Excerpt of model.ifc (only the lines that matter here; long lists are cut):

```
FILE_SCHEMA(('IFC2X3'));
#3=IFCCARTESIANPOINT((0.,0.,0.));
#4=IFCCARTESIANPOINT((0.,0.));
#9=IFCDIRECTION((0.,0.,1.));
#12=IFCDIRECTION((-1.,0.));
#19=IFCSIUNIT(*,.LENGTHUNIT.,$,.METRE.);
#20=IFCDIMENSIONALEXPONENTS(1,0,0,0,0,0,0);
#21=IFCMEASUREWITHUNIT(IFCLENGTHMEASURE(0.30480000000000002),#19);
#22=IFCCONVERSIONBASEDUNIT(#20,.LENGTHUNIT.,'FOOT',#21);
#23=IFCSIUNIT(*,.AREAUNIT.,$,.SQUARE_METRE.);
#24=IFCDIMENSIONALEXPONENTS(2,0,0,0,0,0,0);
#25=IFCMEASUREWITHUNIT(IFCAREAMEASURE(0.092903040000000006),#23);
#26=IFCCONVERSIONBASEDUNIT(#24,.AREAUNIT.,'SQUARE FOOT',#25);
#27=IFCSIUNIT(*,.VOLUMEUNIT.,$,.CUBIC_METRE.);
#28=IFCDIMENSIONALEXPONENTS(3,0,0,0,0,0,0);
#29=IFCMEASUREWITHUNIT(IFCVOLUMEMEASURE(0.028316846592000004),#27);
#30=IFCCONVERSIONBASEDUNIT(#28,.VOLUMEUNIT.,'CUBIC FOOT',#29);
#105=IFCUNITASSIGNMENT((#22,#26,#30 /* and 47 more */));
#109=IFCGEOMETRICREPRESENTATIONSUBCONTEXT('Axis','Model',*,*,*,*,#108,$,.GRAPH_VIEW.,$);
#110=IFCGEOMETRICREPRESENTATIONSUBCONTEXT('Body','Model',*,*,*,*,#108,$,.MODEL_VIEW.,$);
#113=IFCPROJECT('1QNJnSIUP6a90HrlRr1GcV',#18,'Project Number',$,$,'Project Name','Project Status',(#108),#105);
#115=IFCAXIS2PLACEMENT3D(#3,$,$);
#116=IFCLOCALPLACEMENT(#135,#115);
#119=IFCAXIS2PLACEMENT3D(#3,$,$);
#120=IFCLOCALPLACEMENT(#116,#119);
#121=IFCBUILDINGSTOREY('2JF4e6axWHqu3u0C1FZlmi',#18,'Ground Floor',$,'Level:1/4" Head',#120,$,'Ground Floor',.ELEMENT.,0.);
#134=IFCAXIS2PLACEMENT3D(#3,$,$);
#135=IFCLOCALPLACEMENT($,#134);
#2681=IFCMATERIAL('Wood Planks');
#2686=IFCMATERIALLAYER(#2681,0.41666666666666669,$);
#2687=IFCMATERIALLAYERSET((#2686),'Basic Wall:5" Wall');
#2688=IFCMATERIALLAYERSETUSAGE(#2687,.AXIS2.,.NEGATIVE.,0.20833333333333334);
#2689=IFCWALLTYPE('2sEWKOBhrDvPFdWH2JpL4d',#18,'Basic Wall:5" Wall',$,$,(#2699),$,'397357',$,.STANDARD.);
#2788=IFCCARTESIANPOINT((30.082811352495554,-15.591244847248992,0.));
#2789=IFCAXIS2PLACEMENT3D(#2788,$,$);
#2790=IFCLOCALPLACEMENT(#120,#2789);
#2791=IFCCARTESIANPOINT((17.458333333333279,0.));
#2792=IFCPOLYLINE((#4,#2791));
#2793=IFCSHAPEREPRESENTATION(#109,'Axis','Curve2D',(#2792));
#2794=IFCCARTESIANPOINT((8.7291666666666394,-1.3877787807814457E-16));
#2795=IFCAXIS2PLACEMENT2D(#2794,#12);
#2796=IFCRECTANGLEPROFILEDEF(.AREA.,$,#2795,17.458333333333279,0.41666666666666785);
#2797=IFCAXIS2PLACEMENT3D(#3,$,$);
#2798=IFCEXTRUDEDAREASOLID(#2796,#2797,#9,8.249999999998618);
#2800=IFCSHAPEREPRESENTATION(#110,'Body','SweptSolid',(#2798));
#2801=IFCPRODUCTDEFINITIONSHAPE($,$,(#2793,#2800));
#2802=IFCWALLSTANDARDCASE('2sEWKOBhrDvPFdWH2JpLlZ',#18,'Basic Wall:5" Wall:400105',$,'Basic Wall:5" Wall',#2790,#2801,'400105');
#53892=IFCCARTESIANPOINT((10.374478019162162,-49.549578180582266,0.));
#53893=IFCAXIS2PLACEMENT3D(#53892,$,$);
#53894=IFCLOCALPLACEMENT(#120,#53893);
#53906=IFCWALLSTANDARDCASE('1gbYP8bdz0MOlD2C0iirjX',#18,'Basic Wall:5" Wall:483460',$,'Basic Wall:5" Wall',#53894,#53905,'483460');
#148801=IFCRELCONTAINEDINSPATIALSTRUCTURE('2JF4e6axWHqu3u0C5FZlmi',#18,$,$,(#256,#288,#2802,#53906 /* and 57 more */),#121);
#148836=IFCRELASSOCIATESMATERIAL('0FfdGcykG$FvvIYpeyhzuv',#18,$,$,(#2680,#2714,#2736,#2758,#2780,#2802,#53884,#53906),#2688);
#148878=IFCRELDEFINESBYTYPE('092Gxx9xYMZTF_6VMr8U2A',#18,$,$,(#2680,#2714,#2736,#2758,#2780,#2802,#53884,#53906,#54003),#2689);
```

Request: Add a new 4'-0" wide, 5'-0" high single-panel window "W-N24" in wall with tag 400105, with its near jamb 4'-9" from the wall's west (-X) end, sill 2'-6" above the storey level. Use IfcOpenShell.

```python
import numpy as np
import ifcopenshell
import ifcopenshell.api.feature
import ifcopenshell.api.geometry
import ifcopenshell.api.root
import ifcopenshell.api.spatial
import ifcopenshell.api.type
import ifcopenshell.geom
import ifcopenshell.util.element
import ifcopenshell.util.placement
import ifcopenshell.util.representation
import ifcopenshell.util.shape
import ifcopenshell.util.unit

model = ifcopenshell.open("model.ifc")
unit_scale = ifcopenshell.util.unit.calculate_unit_scale(model)
settings = ifcopenshell.geom.settings()


def volume(element):
    """Net volume in cubic metres, openings subtracted."""
    shape = ifcopenshell.geom.create_shape(settings, element)
    return ifcopenshell.util.shape.get_volume(shape.geometry)


wall = model.by_id(2802)
storey = ifcopenshell.util.element.get_container(wall, ifc_class="IfcBuildingStorey")
context = ifcopenshell.util.representation.get_context(model, "Model", "Body", "MODEL_VIEW")
before = volume(wall)

width, height, from_end, sill = 1.2192, 1.524, 1.4478, 0.762  # metres

# The wall runs along its own X axis, and the end named is its -X end.
wall_shape = ifcopenshell.geom.create_shape(settings, wall)
x, y, z = ifcopenshell.util.shape.get_vertices(wall_shape.geometry).T
start = x.min() + from_end
face, thickness = float(y.min()), float(y.max() - y.min())
wall_matrix = ifcopenshell.util.placement.get_local_placement(wall.ObjectPlacement)
level = ifcopenshell.util.placement.get_local_placement(storey.ObjectPlacement)[2, 3]


def in_wall(x, y):
    """Placement at x, y metres in the wall's axes, at sill height."""
    matrix = wall_matrix.copy()
    matrix[:, 3] = wall_matrix @ np.array([x / unit_scale, y / unit_scale, 0.0, 1.0])
    matrix[2, 3] = level + sill / unit_scale
    return matrix


# Opening: a box that overshoots both wall faces by 50 mm.
opening = ifcopenshell.api.root.create_entity(model, ifc_class="IfcOpeningElement")
box = ifcopenshell.api.geometry.add_wall_representation(
    model, context=context, length=width, height=height, thickness=thickness + 0.1
)
ifcopenshell.api.geometry.assign_representation(model, product=opening, representation=box)
ifcopenshell.api.geometry.edit_object_placement(model, product=opening, matrix=in_wall(start, face - 0.05), is_si=False)
ifcopenshell.api.feature.add_feature(model, feature=opening, element=wall)

window = ifcopenshell.api.root.create_entity(model, ifc_class="IfcWindow", name="W-N24")
window.OverallWidth, window.OverallHeight = width / unit_scale, height / unit_scale
body = ifcopenshell.api.geometry.add_window_representation(
    model,
    context=context,
    overall_width=window.OverallWidth,
    overall_height=window.OverallHeight,
    partition_type="SINGLE_PANEL",
)
ifcopenshell.api.geometry.assign_representation(model, product=window, representation=body)
ifcopenshell.api.spatial.assign_container(model, products=[window], relating_structure=storey)
fills = ifcopenshell.api.feature.add_filling(model, opening=opening, element=window)
fills.OwnerHistory = window.OwnerHistory  # required in IFC2X3

# IFC2X3 keeps the operation on the window style.
style = ifcopenshell.api.root.create_entity(model, ifc_class="IfcWindowStyle", name="W-N24")
style.OperationType, style.ConstructionType = "SINGLE_PANEL", "NOTDEFINED"
style.ParameterTakesPrecedence = style.Sizeable = False
ifcopenshell.api.type.assign_type(model, related_objects=[window], relating_type=style)

# Centre the window in the wall's thickness.
ifcopenshell.api.geometry.edit_object_placement(model, product=window, matrix=in_wall(start, face), is_si=False)
window_shape = ifcopenshell.geom.create_shape(settings, window)
depth = ifcopenshell.util.shape.get_vertices(window_shape.geometry)[:, 1]
offset = face + thickness / 2 - (depth.min() + depth.max()) / 2
ifcopenshell.api.geometry.edit_object_placement(model, product=window, matrix=in_wall(start, offset), is_si=False)

after = volume(wall)

print(f"wall volume {before:.3f} -> {after:.3f} m3")

model.write("model_rev.ifc")
```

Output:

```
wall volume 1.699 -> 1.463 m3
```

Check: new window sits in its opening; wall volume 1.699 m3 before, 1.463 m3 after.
